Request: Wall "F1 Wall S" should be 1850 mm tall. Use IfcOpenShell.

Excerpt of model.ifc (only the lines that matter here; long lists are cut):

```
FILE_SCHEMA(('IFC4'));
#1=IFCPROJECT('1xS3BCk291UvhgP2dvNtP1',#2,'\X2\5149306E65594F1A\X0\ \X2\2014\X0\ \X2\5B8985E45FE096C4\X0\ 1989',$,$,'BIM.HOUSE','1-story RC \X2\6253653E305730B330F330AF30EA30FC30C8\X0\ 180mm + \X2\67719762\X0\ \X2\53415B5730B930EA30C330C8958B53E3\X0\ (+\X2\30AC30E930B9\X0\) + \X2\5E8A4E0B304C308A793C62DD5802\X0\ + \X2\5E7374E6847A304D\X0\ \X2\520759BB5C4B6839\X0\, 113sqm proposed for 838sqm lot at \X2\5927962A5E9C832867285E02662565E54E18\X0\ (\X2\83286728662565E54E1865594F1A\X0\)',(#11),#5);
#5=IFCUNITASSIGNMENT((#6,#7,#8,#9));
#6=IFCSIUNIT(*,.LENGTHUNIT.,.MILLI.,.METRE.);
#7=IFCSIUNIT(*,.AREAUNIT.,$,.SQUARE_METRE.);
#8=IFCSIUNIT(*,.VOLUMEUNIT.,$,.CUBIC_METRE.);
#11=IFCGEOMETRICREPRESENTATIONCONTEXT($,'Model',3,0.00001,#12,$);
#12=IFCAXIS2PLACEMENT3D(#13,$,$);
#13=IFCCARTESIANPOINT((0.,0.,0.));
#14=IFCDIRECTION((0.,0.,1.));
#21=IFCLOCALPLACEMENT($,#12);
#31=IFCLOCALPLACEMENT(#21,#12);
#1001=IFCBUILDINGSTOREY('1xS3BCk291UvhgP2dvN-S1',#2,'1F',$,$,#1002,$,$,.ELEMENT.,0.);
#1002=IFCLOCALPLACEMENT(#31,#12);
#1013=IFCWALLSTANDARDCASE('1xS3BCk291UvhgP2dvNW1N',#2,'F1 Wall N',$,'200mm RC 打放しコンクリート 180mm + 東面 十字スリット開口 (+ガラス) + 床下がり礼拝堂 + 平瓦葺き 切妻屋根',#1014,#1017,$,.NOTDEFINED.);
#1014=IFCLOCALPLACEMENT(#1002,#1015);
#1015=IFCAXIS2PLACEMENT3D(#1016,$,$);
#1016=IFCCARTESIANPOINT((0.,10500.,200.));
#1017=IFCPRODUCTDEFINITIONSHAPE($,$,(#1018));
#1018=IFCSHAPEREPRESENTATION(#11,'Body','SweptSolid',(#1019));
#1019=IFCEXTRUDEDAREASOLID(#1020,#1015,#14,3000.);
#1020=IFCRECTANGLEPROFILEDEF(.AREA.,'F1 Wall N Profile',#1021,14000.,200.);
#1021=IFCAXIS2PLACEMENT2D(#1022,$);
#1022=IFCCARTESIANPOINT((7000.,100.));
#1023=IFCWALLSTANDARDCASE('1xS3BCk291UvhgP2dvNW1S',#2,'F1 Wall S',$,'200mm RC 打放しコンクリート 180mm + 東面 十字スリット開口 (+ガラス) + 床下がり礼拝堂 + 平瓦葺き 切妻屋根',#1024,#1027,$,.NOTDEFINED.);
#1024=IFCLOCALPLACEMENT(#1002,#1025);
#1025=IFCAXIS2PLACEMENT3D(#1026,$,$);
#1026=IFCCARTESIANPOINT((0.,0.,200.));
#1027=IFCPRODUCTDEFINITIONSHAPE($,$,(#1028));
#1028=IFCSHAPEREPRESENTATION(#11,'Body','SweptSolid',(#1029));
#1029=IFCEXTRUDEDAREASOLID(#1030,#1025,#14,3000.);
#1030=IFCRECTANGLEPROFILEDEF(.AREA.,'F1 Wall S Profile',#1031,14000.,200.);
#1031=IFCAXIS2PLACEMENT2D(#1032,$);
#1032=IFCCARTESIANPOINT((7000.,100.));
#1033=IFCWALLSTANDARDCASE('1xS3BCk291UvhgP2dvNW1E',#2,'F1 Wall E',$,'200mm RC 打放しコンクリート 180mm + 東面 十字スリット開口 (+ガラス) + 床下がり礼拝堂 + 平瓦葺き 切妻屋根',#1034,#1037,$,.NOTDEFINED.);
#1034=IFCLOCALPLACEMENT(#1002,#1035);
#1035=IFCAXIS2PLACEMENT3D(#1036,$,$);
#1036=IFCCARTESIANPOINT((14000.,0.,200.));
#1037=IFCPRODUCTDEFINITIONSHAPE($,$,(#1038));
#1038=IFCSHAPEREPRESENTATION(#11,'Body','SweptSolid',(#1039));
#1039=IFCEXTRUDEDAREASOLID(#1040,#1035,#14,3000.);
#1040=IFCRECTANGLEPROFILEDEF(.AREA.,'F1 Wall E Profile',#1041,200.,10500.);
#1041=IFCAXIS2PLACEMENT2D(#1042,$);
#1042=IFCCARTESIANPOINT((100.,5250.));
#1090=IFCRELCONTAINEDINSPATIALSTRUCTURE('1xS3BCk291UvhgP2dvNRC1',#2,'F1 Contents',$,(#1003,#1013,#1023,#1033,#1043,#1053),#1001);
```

```python
import ifcopenshell
import ifcopenshell.geom
import ifcopenshell.util.shape
import ifcopenshell.util.unit

model = ifcopenshell.open("model.ifc")
unit_scale = ifcopenshell.util.unit.calculate_unit_scale(model)
settings = ifcopenshell.geom.settings()


def volume(element):
    """Net volume in cubic metres, openings subtracted."""
    shape = ifcopenshell.geom.create_shape(settings, element)
    return ifcopenshell.util.shape.get_volume(shape.geometry)


wall = model.by_guid("1xS3BCk291UvhgP2dvNW1S")
before = volume(wall)

body = next(r for r in wall.Representation.Representations if r.RepresentationIdentifier == "Body")
solid = body.Items[0]
old_height = solid.Depth
solid.Depth = 1.85 / unit_scale
after = volume(wall)

print(f"height {old_height:g} -> {solid.Depth:g}, volume {before:.3f} -> {after:.3f} m3")

model.write("model-out.ifc")
```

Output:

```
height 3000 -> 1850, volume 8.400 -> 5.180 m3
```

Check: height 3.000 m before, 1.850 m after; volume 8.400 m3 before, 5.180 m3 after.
